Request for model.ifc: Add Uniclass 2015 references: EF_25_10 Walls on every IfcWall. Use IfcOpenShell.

First a look at what the model holds.

```python
import ifcopenshell

model = ifcopenshell.open("model.ifc")
print(model.schema)
print("classifications:", [c.Name for c in model.by_type("IfcClassification")])
for ifc_class in ("IfcDoor", "IfcRoof", "IfcStair", "IfcWall", "IfcWindow"):
    print(ifc_class, len(model.by_type(ifc_class)))
```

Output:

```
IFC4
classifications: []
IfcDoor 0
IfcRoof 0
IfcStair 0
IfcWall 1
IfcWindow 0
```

```python
import ifcopenshell
import ifcopenshell.api.classification

model = ifcopenshell.open("model.ifc")

system = ifcopenshell.api.classification.add_classification(model, classification="Uniclass 2015")

codes = {
    "IfcWall": ("EF_25_10", "Walls"),
}
for ifc_class, (code, name) in codes.items():
    products = model.by_type(ifc_class)
    ifcopenshell.api.classification.add_reference(
        model, products=products, classification=system, identification=code, name=name
    )
    print(code, len(products))

model.write("model_edited.ifc")
```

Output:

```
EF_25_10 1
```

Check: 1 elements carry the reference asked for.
